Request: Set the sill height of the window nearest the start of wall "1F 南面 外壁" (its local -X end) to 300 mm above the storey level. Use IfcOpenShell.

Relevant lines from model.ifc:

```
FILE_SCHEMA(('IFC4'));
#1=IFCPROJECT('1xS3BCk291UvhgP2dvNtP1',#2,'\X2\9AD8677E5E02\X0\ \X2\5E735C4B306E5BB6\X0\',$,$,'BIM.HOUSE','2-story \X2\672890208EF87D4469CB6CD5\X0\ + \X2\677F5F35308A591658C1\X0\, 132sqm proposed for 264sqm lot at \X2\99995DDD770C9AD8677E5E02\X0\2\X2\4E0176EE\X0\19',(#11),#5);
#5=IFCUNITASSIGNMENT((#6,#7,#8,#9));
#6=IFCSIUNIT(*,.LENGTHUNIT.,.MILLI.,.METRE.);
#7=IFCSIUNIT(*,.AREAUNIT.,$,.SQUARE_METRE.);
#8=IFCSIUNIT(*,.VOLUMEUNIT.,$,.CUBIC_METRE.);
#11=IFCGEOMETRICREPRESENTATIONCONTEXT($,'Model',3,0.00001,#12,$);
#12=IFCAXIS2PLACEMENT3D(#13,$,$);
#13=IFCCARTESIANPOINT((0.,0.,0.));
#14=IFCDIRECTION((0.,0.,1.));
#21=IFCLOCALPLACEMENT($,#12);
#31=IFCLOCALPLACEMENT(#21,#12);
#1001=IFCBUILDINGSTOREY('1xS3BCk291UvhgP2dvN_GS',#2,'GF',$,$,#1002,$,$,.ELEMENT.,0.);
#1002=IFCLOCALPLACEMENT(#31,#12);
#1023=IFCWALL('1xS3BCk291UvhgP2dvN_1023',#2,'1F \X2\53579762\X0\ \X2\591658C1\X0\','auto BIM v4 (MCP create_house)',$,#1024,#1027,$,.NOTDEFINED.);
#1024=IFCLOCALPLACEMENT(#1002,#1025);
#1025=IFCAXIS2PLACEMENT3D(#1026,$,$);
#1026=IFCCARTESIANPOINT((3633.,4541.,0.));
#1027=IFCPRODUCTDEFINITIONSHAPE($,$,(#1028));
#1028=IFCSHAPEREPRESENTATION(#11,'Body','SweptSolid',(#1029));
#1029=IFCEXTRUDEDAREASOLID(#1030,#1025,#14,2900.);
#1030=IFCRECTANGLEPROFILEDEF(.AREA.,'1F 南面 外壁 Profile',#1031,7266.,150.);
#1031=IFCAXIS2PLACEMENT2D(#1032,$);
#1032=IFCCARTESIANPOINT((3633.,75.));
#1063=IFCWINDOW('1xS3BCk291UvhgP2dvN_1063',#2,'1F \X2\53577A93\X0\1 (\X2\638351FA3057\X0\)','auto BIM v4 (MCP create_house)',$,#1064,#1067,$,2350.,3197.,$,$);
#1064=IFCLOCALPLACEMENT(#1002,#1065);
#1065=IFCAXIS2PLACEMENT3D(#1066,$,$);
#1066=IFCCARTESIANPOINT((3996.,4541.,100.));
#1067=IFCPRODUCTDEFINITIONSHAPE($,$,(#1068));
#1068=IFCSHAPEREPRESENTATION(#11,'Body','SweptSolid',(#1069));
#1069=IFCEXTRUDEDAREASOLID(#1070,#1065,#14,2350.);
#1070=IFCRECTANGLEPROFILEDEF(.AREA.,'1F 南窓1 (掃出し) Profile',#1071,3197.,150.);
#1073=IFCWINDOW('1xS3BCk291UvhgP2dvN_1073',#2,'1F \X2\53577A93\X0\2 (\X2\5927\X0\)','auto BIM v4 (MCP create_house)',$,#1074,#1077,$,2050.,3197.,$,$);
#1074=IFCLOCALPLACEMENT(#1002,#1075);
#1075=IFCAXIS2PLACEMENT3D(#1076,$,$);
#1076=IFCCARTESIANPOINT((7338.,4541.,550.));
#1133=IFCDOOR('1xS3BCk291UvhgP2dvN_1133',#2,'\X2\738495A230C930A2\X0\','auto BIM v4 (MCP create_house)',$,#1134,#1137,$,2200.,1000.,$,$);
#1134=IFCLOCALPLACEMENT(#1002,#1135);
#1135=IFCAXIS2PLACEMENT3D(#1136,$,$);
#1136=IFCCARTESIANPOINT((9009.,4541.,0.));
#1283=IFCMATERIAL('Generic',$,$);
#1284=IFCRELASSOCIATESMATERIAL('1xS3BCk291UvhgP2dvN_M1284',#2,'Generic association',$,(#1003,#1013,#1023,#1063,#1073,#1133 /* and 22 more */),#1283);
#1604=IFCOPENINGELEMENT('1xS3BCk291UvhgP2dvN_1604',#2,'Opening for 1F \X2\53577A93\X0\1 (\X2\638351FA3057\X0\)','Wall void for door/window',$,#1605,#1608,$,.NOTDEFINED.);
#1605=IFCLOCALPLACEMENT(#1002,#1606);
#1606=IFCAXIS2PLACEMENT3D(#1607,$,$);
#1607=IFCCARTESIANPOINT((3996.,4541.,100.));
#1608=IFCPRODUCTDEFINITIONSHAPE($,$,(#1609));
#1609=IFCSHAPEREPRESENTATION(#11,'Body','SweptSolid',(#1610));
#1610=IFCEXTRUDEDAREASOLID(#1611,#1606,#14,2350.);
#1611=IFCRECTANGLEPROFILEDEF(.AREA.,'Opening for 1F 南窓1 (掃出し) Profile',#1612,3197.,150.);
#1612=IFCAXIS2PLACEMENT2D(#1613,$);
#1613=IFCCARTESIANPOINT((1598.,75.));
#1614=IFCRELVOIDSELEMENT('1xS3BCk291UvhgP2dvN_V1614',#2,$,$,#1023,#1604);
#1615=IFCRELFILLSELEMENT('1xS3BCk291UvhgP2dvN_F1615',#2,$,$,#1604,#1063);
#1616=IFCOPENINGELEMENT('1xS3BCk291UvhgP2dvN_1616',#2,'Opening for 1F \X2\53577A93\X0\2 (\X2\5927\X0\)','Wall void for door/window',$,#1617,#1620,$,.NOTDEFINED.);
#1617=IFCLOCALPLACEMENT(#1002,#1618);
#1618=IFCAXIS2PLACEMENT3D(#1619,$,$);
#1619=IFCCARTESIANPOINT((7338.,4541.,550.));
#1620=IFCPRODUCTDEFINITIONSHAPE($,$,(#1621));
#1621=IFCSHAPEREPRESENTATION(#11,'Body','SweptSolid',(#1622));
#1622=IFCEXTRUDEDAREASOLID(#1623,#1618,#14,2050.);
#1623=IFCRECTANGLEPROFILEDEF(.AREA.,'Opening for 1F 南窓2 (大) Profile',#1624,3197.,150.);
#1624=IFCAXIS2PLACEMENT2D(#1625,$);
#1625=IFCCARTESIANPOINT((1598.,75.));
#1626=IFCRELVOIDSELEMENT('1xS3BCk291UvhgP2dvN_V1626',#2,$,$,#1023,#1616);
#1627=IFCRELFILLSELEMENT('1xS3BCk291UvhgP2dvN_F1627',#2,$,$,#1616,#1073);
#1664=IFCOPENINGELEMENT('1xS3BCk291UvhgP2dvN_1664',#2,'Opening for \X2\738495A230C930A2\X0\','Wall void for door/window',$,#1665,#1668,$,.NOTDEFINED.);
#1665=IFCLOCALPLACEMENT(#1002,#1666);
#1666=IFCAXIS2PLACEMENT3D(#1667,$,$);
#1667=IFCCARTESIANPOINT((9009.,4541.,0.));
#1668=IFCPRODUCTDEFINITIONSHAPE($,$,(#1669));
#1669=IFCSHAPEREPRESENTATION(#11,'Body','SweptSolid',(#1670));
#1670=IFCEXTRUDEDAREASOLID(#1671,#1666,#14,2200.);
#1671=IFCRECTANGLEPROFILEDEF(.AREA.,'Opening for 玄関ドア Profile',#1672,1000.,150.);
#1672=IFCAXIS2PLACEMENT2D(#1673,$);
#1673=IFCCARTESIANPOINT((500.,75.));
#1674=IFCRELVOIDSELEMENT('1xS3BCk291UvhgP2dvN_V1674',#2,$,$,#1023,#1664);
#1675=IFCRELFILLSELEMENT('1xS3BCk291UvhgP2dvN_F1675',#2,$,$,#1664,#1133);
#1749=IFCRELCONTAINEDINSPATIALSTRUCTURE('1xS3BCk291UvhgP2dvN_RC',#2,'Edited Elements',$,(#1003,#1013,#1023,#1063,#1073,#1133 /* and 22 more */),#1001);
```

```python
import numpy as np
import ifcopenshell
import ifcopenshell.api.geometry
import ifcopenshell.geom
import ifcopenshell.util.element
import ifcopenshell.util.placement
import ifcopenshell.util.shape
import ifcopenshell.util.unit

model = ifcopenshell.open("model.ifc")
unit_scale = ifcopenshell.util.unit.calculate_unit_scale(model)

window = model.by_guid("1xS3BCk291UvhgP2dvN_1063")
opening = window.FillsVoids[0].RelatingOpeningElement
storey = ifcopenshell.util.element.get_container(window, ifc_class="IfcBuildingStorey")
level = ifcopenshell.util.placement.get_local_placement(storey.ObjectPlacement)[2, 3]

# The opening's origin need not be at the sill, so measure its lowest point.
shape = ifcopenshell.geom.create_shape(ifcopenshell.geom.settings(), opening)
bottom = ifcopenshell.util.shape.get_shape_bottom_elevation(shape, shape.geometry) / unit_scale
dz = level + 0.3 / unit_scale - bottom

shift = np.array([0.0, 0.0, dz])
# The window is not placed relative to its opening, so move both.
for product in (opening, window):
    matrix = ifcopenshell.util.placement.get_local_placement(product.ObjectPlacement)
    matrix[:3, 3] += shift
    ifcopenshell.api.geometry.edit_object_placement(model, product=product, matrix=matrix, is_si=False)

print(f"moved by {dz * unit_scale:+.3f} m")

model.write("model_edited.ifc")
```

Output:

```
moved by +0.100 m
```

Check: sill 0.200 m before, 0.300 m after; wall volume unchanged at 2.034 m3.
